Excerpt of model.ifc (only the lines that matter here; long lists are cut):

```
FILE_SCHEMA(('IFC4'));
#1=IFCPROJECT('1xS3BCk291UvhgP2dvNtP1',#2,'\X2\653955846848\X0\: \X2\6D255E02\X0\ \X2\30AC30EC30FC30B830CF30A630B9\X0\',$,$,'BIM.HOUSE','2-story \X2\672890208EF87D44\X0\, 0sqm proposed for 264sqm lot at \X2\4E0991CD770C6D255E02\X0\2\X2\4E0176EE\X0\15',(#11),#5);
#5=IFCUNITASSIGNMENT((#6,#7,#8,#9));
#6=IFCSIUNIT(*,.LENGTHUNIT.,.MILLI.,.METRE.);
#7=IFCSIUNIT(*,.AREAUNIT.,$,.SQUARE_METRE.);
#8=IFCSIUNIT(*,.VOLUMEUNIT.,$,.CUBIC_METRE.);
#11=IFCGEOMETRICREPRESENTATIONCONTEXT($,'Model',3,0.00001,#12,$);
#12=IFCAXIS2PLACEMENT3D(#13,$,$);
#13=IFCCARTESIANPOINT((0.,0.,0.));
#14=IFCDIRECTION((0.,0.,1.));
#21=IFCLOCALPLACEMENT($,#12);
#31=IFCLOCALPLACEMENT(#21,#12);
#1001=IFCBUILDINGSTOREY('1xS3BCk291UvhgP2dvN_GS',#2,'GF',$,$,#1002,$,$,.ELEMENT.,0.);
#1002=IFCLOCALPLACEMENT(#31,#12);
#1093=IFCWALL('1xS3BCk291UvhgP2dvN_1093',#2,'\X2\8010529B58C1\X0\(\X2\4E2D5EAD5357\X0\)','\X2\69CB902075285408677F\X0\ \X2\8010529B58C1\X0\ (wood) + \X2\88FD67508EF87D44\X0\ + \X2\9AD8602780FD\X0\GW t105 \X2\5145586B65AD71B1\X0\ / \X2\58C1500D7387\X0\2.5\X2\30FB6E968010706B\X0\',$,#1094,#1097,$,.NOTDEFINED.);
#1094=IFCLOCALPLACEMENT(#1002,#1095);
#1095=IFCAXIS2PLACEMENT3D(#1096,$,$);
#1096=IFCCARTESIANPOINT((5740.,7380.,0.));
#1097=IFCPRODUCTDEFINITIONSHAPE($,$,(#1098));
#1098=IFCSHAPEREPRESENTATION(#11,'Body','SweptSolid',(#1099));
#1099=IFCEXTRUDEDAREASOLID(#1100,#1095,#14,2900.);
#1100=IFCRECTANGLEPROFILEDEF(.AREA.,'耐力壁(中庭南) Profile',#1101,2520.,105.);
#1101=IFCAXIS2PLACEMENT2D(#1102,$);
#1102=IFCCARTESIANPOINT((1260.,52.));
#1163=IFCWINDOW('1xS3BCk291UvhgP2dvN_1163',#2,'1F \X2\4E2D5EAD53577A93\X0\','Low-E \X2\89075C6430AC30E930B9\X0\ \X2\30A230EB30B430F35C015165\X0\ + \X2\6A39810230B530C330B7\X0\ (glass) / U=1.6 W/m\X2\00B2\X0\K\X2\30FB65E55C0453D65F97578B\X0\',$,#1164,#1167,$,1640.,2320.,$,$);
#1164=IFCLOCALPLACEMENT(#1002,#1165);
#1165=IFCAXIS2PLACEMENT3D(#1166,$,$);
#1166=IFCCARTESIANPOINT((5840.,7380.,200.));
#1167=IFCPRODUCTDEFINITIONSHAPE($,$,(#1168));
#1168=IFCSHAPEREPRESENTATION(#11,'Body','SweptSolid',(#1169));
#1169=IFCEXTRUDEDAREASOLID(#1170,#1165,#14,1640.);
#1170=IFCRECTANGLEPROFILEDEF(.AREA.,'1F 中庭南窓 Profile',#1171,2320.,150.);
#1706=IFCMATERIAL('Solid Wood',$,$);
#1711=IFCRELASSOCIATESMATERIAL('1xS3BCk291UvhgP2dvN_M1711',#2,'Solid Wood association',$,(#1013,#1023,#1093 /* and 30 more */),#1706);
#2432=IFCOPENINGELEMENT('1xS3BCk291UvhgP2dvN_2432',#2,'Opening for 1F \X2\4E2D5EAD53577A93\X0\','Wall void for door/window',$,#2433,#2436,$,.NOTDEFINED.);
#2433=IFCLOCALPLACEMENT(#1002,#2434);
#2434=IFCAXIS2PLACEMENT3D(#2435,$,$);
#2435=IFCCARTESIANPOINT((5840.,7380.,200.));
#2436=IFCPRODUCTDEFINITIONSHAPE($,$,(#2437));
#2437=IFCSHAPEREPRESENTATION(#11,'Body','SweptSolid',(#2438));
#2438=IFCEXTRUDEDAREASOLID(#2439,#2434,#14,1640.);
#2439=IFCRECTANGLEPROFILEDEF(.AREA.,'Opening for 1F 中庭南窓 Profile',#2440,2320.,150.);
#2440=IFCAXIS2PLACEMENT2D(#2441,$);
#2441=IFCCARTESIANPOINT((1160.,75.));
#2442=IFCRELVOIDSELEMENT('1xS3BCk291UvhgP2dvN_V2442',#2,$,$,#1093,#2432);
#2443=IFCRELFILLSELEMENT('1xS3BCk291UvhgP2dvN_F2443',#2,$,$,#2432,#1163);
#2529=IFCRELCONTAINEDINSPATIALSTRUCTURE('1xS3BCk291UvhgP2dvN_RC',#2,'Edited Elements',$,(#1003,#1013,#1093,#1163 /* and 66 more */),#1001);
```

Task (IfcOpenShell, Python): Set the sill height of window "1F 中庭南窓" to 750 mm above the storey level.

```python
import numpy as np
import ifcopenshell
import ifcopenshell.api.geometry
import ifcopenshell.geom
import ifcopenshell.util.element
import ifcopenshell.util.placement
import ifcopenshell.util.shape
import ifcopenshell.util.unit

model = ifcopenshell.open("model.ifc")
unit_scale = ifcopenshell.util.unit.calculate_unit_scale(model)

window = model.by_guid("1xS3BCk291UvhgP2dvN_1163")
opening = window.FillsVoids[0].RelatingOpeningElement
storey = ifcopenshell.util.element.get_container(window, ifc_class="IfcBuildingStorey")
level = ifcopenshell.util.placement.get_local_placement(storey.ObjectPlacement)[2, 3]

# The opening's origin need not be at the sill, so measure its lowest point.
shape = ifcopenshell.geom.create_shape(ifcopenshell.geom.settings(), opening)
bottom = ifcopenshell.util.shape.get_shape_bottom_elevation(shape, shape.geometry) / unit_scale
dz = level + 0.75 / unit_scale - bottom

shift = np.array([0.0, 0.0, dz])
# The window is not placed relative to its opening, so move both.
for product in (opening, window):
    matrix = ifcopenshell.util.placement.get_local_placement(product.ObjectPlacement)
    matrix[:3, 3] += shift
    ifcopenshell.api.geometry.edit_object_placement(model, product=product, matrix=matrix, is_si=False)

print(f"moved by {dz * unit_scale:+.3f} m")

model.write("model_edited.ifc")
```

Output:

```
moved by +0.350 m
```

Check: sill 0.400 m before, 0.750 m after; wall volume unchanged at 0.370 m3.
